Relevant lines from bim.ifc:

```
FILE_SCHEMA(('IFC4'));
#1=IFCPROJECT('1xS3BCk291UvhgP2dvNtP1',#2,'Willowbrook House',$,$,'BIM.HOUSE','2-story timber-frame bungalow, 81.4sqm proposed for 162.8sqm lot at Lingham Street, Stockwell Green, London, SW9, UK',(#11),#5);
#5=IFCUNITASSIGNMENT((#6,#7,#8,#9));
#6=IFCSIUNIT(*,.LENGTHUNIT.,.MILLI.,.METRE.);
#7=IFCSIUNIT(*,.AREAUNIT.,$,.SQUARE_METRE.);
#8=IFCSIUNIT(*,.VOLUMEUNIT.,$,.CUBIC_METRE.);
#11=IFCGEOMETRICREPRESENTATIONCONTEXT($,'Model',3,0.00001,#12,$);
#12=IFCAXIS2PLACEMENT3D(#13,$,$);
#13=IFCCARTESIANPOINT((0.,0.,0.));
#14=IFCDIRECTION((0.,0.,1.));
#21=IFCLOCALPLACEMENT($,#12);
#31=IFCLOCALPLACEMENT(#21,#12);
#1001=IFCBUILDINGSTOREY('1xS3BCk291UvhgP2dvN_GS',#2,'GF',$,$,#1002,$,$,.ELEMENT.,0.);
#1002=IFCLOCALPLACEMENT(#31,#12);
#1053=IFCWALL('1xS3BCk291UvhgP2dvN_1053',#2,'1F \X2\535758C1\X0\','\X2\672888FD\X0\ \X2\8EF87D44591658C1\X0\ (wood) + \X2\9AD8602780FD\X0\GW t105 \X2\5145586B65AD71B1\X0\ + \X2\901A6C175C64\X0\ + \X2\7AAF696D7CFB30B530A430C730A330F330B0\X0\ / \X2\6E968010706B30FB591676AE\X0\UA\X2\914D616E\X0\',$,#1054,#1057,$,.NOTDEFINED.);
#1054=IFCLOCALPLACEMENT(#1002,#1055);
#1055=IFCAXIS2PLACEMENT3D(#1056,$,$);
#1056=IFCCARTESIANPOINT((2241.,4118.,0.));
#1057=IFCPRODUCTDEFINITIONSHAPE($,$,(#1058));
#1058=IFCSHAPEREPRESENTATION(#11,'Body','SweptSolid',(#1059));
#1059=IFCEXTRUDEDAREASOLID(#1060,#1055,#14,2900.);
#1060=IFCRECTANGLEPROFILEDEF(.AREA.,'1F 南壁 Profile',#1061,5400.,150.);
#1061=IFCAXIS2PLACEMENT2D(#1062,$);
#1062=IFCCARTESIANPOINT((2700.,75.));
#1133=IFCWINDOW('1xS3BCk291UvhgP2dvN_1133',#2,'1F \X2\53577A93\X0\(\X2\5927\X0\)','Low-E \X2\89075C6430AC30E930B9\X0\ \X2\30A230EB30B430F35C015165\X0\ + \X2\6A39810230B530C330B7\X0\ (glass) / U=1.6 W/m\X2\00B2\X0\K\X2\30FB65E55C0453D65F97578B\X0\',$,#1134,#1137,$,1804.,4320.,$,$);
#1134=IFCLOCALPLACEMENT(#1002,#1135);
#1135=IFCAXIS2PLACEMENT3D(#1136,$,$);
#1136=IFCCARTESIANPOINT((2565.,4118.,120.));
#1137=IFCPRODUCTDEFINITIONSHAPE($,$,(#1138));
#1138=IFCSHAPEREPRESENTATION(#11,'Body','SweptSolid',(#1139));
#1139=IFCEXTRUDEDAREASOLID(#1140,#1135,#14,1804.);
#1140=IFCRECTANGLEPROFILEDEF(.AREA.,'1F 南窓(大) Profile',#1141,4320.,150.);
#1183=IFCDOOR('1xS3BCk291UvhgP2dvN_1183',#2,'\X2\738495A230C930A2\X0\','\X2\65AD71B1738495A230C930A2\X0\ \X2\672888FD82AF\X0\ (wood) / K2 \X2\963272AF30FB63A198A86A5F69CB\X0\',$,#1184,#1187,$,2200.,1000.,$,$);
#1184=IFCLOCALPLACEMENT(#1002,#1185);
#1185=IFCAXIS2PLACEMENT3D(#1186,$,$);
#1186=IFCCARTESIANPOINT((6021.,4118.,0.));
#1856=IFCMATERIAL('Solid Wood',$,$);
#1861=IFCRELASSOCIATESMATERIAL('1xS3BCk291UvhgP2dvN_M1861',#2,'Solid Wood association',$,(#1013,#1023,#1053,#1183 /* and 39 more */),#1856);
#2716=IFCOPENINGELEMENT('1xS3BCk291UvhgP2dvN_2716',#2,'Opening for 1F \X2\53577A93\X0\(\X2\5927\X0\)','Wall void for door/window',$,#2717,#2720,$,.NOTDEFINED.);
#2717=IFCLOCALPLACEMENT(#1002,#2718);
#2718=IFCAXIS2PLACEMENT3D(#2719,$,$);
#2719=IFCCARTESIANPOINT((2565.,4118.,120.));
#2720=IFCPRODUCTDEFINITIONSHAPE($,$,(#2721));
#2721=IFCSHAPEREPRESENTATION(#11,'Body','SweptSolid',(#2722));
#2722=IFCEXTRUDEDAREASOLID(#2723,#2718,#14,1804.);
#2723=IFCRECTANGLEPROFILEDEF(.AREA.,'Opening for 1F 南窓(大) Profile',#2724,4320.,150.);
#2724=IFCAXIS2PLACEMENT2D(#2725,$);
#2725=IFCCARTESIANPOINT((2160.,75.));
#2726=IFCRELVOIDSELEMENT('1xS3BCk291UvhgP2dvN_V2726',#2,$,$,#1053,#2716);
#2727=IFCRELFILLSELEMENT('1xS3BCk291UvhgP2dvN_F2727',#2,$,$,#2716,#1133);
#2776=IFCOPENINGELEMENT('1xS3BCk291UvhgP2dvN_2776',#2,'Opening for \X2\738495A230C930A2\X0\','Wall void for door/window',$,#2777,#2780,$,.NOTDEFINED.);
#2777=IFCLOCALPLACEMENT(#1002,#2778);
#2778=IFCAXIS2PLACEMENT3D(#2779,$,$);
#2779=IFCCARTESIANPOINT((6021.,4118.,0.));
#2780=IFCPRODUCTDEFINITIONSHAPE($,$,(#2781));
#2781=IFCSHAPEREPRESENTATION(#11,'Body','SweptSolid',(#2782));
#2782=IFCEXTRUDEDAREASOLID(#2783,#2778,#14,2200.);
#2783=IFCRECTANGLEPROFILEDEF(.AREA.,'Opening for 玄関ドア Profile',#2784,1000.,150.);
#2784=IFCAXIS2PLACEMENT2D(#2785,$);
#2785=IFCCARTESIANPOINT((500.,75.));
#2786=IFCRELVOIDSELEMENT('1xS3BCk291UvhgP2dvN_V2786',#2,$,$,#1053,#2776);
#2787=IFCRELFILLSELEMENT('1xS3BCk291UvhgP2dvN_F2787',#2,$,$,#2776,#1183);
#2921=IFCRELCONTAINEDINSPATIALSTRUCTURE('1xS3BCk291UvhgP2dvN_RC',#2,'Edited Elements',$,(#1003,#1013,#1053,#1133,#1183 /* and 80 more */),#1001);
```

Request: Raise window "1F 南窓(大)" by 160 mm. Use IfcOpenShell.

```python
import numpy as np
import ifcopenshell
import ifcopenshell.api.geometry
import ifcopenshell.util.placement
import ifcopenshell.util.unit

model = ifcopenshell.open("bim.ifc")
unit_scale = ifcopenshell.util.unit.calculate_unit_scale(model)

window = model.by_guid("1xS3BCk291UvhgP2dvN_1133")
opening = window.FillsVoids[0].RelatingOpeningElement
dz = 160.0

shift = np.array([0.0, 0.0, dz])
# The window is not placed relative to its opening, so move both.
for product in (opening, window):
    matrix = ifcopenshell.util.placement.get_local_placement(product.ObjectPlacement)
    matrix[:3, 3] += shift
    ifcopenshell.api.geometry.edit_object_placement(model, product=product, matrix=matrix, is_si=False)

print(f"moved by {dz * unit_scale:+.3f} m")

model.write("bim_updated.ifc")
```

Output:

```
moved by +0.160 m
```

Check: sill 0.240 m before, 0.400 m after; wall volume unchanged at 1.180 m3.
